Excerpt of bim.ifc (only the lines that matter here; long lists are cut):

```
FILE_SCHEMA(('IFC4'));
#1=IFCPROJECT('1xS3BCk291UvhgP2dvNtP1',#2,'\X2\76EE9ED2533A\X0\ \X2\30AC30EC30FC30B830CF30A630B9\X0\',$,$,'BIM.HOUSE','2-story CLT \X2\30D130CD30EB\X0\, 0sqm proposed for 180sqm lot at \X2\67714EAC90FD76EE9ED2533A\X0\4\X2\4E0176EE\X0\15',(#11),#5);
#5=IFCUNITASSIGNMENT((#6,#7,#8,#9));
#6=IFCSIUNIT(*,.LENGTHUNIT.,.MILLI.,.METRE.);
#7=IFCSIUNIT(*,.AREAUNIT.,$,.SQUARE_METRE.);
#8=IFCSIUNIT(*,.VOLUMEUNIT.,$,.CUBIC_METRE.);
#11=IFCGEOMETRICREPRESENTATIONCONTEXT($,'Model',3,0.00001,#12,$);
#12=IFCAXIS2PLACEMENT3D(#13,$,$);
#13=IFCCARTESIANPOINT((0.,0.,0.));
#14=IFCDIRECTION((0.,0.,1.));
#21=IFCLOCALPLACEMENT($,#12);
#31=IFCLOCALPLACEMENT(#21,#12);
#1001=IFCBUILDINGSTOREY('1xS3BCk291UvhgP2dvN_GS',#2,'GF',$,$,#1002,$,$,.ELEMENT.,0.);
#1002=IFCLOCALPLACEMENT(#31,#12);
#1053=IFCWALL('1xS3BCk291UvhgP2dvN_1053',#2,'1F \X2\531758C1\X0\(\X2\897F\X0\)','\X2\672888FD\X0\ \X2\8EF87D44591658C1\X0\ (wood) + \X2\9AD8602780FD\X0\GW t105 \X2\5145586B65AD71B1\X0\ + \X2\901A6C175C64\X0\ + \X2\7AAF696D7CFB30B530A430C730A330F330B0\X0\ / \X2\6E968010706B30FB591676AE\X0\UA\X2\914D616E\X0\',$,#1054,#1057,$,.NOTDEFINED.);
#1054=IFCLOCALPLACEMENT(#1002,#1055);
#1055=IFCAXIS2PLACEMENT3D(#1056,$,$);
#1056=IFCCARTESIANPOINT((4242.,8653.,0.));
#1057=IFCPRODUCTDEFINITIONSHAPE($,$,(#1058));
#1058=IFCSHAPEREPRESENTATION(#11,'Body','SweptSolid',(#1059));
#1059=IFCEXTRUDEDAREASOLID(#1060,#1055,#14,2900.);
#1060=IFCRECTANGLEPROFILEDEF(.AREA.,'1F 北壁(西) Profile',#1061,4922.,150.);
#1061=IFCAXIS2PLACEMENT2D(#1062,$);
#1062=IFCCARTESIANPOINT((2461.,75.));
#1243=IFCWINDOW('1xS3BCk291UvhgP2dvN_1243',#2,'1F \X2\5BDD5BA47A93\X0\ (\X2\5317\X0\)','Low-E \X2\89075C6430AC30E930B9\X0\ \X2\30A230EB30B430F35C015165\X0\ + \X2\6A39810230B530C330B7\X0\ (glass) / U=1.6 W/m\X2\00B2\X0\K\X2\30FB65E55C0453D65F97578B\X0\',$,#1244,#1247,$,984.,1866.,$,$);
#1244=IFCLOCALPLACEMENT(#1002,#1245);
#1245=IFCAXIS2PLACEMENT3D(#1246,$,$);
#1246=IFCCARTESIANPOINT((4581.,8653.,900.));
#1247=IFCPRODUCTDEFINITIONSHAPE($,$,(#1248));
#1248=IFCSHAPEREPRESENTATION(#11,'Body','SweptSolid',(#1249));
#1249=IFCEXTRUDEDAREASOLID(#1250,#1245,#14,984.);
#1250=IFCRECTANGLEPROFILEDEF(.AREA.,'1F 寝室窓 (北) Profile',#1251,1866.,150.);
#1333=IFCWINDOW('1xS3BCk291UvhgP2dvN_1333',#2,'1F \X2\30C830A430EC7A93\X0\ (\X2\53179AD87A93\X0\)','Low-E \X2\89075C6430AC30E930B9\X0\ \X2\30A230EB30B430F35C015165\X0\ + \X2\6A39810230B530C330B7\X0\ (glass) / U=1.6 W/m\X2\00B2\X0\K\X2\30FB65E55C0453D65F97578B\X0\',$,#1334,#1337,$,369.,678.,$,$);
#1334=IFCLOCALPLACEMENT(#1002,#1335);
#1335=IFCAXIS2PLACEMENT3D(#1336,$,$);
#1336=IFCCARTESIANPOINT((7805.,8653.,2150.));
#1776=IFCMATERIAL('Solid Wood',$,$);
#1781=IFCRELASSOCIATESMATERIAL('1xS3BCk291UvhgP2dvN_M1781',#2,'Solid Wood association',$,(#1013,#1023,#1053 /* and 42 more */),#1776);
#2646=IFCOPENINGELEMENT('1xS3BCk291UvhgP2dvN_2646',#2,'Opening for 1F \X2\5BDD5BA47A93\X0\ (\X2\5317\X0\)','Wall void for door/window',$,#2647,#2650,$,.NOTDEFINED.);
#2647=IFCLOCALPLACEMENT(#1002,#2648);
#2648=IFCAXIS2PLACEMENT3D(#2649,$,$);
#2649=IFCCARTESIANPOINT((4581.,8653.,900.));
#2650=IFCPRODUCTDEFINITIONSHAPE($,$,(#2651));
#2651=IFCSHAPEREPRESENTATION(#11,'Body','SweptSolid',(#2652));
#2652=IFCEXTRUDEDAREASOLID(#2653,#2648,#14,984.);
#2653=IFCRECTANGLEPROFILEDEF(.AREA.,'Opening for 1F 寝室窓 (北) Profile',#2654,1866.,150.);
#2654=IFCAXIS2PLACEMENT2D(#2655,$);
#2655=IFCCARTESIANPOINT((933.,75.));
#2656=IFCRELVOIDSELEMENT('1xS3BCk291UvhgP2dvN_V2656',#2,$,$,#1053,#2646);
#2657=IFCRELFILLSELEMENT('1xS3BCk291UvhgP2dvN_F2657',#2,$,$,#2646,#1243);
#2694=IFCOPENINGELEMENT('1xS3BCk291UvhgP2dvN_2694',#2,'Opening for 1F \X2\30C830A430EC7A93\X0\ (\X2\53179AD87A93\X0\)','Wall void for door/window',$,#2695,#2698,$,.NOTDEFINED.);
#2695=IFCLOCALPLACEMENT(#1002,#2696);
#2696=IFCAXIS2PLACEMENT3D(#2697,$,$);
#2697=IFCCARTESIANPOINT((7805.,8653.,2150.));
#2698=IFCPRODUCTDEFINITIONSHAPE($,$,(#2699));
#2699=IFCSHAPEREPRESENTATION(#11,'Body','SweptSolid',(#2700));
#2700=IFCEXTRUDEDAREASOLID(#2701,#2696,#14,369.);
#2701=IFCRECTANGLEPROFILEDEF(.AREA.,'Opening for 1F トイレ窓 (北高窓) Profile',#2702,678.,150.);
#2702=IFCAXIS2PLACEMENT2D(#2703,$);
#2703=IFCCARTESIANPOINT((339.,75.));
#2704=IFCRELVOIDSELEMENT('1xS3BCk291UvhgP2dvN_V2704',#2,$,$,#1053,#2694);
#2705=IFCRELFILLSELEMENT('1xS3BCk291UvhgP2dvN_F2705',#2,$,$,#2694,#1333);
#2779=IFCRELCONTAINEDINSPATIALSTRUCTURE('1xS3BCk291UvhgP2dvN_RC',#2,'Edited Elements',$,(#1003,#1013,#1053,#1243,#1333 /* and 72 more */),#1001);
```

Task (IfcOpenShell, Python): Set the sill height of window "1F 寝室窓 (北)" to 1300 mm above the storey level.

```python
import numpy as np
import ifcopenshell
import ifcopenshell.api.geometry
import ifcopenshell.geom
import ifcopenshell.util.element
import ifcopenshell.util.placement
import ifcopenshell.util.shape
import ifcopenshell.util.unit

model = ifcopenshell.open("bim.ifc")
unit_scale = ifcopenshell.util.unit.calculate_unit_scale(model)

window = model.by_guid("1xS3BCk291UvhgP2dvN_1243")
opening = window.FillsVoids[0].RelatingOpeningElement
storey = ifcopenshell.util.element.get_container(window, ifc_class="IfcBuildingStorey")
level = ifcopenshell.util.placement.get_local_placement(storey.ObjectPlacement)[2, 3]

# The opening's origin need not be at the sill, so measure its lowest point.
shape = ifcopenshell.geom.create_shape(ifcopenshell.geom.settings(), opening)
bottom = ifcopenshell.util.shape.get_shape_bottom_elevation(shape, shape.geometry) / unit_scale
dz = level + 1.3 / unit_scale - bottom

shift = np.array([0.0, 0.0, dz])
# The window is not placed relative to its opening, so move both.
for product in (opening, window):
    matrix = ifcopenshell.util.placement.get_local_placement(product.ObjectPlacement)
    matrix[:3, 3] += shift
    ifcopenshell.api.geometry.edit_object_placement(model, product=product, matrix=matrix, is_si=False)

print(f"moved by {dz * unit_scale:+.3f} m")

model.write("bim_updated.ifc")
```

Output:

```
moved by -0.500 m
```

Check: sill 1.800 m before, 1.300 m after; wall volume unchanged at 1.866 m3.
